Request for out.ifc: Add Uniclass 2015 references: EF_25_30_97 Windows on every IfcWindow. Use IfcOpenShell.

First a look at what the model holds.

```python
import ifcopenshell

model = ifcopenshell.open("out.ifc")
print(model.schema)
print("classifications:", [c.Name for c in model.by_type("IfcClassification")])
for ifc_class in ("IfcDoor", "IfcRoof", "IfcStair", "IfcWall", "IfcWindow"):
    print(ifc_class, len(model.by_type(ifc_class)))
```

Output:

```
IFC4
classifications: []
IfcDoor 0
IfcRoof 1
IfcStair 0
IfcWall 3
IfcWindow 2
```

```python
import ifcopenshell
import ifcopenshell.api.classification

model = ifcopenshell.open("out.ifc")

system = ifcopenshell.api.classification.add_classification(model, classification="Uniclass 2015")

codes = {
    "IfcWindow": ("EF_25_30_97", "Windows"),
}
for ifc_class, (code, name) in codes.items():
    products = model.by_type(ifc_class)
    ifcopenshell.api.classification.add_reference(
        model, products=products, classification=system, identification=code, name=name
    )
    print(code, len(products))

model.write("out_v2.ifc")
```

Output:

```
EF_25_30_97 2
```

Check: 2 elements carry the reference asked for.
